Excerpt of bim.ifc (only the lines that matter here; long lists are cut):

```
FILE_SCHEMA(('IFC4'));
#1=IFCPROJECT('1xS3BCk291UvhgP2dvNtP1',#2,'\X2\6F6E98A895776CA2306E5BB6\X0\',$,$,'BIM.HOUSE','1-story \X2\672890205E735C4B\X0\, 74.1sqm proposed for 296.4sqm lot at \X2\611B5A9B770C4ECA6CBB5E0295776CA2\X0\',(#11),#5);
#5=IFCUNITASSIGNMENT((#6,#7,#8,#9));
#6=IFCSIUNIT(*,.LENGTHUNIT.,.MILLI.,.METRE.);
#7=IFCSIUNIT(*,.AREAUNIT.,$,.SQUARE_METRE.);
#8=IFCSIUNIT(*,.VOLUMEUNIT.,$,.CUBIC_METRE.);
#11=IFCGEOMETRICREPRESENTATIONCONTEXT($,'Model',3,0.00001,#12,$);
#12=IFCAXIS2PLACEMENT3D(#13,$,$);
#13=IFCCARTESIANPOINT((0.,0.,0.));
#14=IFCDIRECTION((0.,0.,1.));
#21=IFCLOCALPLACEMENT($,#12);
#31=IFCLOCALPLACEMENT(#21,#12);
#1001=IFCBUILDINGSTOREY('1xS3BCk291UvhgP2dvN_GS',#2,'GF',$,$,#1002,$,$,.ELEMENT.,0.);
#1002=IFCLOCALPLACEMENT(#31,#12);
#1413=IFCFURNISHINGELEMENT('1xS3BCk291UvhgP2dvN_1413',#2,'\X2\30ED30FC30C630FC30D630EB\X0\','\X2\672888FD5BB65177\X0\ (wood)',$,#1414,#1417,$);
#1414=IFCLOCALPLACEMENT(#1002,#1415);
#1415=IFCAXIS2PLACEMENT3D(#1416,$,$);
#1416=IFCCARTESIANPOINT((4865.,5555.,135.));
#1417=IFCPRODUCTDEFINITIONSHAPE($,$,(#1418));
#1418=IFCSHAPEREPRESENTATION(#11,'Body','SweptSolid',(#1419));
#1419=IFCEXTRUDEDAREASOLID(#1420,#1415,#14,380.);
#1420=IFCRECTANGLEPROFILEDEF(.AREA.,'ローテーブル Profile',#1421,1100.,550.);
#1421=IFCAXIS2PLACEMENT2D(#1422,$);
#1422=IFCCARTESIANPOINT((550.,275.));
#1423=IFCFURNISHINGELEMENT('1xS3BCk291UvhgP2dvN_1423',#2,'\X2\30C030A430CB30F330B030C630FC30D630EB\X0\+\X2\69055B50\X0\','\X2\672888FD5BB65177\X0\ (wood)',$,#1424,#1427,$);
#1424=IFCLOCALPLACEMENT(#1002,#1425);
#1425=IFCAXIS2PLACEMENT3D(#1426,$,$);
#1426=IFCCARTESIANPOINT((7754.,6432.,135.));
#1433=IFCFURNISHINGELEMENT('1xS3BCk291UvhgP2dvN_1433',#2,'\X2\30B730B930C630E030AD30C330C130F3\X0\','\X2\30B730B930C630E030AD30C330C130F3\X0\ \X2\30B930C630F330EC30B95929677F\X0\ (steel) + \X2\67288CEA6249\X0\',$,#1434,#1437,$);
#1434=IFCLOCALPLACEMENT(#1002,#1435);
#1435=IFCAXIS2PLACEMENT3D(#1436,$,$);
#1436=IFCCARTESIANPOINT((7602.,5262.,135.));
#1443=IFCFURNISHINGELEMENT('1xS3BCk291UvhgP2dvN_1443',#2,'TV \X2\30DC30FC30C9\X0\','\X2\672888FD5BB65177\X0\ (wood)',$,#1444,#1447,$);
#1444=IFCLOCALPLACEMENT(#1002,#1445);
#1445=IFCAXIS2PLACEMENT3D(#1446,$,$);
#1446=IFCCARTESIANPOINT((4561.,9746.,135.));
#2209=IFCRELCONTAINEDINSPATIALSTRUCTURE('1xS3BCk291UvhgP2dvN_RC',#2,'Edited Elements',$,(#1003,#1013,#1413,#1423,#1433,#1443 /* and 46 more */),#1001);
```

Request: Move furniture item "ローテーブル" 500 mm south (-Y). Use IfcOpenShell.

```python
import ifcopenshell
import ifcopenshell.api.geometry
import ifcopenshell.util.placement
import ifcopenshell.util.unit

model = ifcopenshell.open("bim.ifc")
unit_scale = ifcopenshell.util.unit.calculate_unit_scale(model)

item = model.by_id(1413)
matrix = ifcopenshell.util.placement.get_local_placement(item.ObjectPlacement)
matrix[1, 3] -= 0.5 / unit_scale
ifcopenshell.api.geometry.edit_object_placement(model, product=item, matrix=matrix, is_si=False)

print(ifcopenshell.util.placement.get_local_placement(item.ObjectPlacement).round(3) + 0.0)

model.write("bim_rev.ifc")
```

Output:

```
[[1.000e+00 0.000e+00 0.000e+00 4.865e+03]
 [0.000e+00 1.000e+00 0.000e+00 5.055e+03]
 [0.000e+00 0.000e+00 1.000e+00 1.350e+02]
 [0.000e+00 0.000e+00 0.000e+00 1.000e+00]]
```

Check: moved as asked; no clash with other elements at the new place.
